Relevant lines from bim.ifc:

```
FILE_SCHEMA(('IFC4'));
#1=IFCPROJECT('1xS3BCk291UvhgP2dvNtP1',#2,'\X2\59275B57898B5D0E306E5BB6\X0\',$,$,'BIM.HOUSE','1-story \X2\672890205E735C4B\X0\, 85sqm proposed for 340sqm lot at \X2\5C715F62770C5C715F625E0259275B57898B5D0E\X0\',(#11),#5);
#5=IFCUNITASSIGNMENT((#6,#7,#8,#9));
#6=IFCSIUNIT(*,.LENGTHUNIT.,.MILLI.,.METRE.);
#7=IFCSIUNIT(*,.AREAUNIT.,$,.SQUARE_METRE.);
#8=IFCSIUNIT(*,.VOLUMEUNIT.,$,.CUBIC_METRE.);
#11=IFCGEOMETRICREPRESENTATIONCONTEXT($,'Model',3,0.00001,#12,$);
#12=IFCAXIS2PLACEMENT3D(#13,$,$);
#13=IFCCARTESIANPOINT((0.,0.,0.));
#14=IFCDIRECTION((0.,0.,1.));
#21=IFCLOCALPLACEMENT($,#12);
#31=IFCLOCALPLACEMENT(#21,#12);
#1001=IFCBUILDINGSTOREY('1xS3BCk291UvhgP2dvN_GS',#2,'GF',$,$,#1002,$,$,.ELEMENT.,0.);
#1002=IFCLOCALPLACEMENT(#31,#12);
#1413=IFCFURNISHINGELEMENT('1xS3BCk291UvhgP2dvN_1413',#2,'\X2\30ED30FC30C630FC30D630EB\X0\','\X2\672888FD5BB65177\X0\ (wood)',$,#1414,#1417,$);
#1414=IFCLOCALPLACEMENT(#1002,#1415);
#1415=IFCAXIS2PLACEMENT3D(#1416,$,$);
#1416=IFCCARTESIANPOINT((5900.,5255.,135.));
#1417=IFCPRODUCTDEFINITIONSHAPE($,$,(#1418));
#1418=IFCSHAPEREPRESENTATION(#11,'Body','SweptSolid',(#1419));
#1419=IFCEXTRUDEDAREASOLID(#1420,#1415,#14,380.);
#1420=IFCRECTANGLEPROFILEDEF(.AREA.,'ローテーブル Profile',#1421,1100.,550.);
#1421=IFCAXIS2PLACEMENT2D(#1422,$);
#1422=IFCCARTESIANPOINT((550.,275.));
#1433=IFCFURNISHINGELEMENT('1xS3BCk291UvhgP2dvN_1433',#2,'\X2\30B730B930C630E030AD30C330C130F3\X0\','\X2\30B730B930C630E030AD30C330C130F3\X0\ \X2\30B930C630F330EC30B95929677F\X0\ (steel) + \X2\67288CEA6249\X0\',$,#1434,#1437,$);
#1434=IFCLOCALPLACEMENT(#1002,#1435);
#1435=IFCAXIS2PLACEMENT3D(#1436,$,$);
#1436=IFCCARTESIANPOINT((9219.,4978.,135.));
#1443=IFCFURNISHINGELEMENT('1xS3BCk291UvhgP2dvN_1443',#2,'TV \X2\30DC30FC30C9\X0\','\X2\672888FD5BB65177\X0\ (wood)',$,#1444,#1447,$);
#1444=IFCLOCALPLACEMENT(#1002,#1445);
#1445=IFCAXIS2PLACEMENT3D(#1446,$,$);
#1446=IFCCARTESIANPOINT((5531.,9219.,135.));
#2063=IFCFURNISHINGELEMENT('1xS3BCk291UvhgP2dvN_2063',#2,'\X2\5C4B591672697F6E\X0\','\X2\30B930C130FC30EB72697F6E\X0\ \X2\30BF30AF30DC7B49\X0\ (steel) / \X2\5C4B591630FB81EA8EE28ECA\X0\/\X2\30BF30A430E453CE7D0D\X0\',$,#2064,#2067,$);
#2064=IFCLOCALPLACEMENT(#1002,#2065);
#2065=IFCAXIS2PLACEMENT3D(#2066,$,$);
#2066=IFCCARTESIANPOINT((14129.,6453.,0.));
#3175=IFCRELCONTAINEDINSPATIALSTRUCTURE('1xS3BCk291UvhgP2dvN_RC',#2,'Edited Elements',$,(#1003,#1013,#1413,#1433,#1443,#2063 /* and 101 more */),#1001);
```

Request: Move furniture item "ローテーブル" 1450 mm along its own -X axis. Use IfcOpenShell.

```python
import ifcopenshell
import ifcopenshell.api.geometry
import ifcopenshell.util.placement

model = ifcopenshell.open("bim.ifc")

item = model.by_guid("1xS3BCk291UvhgP2dvN_1413")
matrix = ifcopenshell.util.placement.get_local_placement(item.ObjectPlacement)
matrix[:3, 3] -= matrix[:3, 0] * 1450.0
ifcopenshell.api.geometry.edit_object_placement(model, product=item, matrix=matrix, is_si=False)

print(ifcopenshell.util.placement.get_local_placement(item.ObjectPlacement).round(3) + 0.0)

model.write("bim_v2.ifc")
```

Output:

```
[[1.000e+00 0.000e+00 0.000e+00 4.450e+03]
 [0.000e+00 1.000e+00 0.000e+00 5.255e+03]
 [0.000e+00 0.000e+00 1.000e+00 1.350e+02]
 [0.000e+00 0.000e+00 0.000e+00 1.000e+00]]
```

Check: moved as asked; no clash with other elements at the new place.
